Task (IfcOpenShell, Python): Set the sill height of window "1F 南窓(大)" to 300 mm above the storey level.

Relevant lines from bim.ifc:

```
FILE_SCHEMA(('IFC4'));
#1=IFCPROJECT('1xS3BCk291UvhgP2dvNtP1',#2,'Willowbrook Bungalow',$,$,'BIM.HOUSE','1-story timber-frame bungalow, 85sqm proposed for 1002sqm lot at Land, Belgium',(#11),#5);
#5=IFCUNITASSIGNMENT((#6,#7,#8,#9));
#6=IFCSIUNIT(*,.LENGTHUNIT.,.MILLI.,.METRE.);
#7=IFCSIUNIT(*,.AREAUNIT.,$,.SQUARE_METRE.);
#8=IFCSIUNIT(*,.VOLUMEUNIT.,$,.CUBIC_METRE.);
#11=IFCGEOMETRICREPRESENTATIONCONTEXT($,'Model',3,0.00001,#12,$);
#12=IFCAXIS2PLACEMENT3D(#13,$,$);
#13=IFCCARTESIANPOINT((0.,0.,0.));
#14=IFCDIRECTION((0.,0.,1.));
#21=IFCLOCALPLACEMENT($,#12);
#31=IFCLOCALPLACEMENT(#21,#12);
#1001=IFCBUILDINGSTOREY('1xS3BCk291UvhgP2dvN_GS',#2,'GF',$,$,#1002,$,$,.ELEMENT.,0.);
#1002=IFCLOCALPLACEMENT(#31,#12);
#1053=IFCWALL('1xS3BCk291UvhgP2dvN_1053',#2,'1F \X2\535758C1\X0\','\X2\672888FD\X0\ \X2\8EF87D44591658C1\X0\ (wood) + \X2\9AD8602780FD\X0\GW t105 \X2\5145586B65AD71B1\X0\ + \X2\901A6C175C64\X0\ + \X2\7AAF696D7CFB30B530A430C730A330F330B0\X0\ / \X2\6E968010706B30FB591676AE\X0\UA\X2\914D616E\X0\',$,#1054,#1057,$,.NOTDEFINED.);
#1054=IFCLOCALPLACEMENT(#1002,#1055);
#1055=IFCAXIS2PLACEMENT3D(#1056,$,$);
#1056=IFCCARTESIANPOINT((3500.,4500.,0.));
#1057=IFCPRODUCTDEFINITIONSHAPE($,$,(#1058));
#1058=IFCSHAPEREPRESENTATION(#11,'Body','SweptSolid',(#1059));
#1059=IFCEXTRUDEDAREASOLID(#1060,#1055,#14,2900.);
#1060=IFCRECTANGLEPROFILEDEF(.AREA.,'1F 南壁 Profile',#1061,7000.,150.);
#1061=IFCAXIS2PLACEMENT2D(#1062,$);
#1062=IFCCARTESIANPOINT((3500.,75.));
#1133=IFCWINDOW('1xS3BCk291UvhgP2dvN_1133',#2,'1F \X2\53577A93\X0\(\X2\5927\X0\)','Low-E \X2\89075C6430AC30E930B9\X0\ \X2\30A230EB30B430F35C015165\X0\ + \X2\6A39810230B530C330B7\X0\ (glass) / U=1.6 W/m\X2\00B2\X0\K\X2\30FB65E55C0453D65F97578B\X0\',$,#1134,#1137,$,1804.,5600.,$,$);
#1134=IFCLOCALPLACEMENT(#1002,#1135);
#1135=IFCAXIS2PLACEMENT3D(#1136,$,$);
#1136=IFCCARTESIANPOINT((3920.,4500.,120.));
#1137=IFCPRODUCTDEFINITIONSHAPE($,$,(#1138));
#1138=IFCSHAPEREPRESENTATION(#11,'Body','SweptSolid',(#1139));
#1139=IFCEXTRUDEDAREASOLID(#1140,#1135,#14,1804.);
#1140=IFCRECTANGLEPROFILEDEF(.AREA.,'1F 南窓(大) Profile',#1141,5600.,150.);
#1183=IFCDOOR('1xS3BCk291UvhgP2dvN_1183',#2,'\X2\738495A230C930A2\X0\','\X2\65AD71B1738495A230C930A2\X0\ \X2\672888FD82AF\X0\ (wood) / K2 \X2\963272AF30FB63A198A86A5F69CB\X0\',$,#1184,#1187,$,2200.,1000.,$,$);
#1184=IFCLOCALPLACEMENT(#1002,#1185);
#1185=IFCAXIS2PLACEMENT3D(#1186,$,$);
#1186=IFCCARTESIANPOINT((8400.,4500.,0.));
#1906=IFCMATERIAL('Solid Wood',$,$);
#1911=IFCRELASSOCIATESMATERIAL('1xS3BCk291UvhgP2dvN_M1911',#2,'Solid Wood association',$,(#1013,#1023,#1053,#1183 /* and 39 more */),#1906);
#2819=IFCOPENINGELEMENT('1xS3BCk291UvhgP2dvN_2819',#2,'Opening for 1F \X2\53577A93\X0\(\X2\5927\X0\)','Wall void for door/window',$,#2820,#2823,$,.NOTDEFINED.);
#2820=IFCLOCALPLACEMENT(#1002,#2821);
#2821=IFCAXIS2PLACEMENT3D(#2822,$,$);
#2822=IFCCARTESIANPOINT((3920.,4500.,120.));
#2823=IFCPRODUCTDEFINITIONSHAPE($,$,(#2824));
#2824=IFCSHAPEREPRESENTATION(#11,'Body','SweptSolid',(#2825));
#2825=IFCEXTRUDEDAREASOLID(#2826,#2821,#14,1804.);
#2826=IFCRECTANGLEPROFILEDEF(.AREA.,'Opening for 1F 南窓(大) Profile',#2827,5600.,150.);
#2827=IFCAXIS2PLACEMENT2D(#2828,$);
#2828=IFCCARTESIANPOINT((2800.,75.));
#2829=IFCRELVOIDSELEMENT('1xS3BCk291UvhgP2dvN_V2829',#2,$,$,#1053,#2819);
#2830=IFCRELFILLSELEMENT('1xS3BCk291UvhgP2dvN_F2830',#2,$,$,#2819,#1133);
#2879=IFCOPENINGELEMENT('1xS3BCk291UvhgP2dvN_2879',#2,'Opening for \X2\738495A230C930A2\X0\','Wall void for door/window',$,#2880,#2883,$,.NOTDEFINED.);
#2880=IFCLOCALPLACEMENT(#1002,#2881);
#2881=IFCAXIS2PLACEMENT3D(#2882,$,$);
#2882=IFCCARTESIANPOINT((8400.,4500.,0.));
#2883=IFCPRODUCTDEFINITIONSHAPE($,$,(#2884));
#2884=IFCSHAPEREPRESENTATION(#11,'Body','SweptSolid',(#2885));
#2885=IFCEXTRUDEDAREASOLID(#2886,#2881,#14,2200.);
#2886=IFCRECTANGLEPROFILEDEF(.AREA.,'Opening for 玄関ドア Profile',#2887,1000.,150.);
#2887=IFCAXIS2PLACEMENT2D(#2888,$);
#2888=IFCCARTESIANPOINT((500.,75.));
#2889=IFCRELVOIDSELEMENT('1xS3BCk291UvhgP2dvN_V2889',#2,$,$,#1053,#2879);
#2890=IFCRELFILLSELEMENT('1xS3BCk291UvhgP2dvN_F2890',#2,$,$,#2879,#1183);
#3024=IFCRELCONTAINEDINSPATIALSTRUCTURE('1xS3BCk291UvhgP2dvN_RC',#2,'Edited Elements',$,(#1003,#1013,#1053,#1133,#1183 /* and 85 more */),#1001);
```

```python
import numpy as np
import ifcopenshell
import ifcopenshell.api.geometry
import ifcopenshell.geom
import ifcopenshell.util.element
import ifcopenshell.util.placement
import ifcopenshell.util.shape
import ifcopenshell.util.unit

model = ifcopenshell.open("bim.ifc")
unit_scale = ifcopenshell.util.unit.calculate_unit_scale(model)

window = model.by_guid("1xS3BCk291UvhgP2dvN_1133")
opening = window.FillsVoids[0].RelatingOpeningElement
storey = ifcopenshell.util.element.get_container(window, ifc_class="IfcBuildingStorey")
level = ifcopenshell.util.placement.get_local_placement(storey.ObjectPlacement)[2, 3]

# The opening's origin need not be at the sill, so measure its lowest point.
shape = ifcopenshell.geom.create_shape(ifcopenshell.geom.settings(), opening)
bottom = ifcopenshell.util.shape.get_shape_bottom_elevation(shape, shape.geometry) / unit_scale
dz = level + 0.3 / unit_scale - bottom

shift = np.array([0.0, 0.0, dz])
# The window is not placed relative to its opening, so move both.
for product in (opening, window):
    matrix = ifcopenshell.util.placement.get_local_placement(product.ObjectPlacement)
    matrix[:3, 3] += shift
    ifcopenshell.api.geometry.edit_object_placement(model, product=product, matrix=matrix, is_si=False)

print(f"moved by {dz * unit_scale:+.3f} m")

model.write("bim_updated.ifc")
```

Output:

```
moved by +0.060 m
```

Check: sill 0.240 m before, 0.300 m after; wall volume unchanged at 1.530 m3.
